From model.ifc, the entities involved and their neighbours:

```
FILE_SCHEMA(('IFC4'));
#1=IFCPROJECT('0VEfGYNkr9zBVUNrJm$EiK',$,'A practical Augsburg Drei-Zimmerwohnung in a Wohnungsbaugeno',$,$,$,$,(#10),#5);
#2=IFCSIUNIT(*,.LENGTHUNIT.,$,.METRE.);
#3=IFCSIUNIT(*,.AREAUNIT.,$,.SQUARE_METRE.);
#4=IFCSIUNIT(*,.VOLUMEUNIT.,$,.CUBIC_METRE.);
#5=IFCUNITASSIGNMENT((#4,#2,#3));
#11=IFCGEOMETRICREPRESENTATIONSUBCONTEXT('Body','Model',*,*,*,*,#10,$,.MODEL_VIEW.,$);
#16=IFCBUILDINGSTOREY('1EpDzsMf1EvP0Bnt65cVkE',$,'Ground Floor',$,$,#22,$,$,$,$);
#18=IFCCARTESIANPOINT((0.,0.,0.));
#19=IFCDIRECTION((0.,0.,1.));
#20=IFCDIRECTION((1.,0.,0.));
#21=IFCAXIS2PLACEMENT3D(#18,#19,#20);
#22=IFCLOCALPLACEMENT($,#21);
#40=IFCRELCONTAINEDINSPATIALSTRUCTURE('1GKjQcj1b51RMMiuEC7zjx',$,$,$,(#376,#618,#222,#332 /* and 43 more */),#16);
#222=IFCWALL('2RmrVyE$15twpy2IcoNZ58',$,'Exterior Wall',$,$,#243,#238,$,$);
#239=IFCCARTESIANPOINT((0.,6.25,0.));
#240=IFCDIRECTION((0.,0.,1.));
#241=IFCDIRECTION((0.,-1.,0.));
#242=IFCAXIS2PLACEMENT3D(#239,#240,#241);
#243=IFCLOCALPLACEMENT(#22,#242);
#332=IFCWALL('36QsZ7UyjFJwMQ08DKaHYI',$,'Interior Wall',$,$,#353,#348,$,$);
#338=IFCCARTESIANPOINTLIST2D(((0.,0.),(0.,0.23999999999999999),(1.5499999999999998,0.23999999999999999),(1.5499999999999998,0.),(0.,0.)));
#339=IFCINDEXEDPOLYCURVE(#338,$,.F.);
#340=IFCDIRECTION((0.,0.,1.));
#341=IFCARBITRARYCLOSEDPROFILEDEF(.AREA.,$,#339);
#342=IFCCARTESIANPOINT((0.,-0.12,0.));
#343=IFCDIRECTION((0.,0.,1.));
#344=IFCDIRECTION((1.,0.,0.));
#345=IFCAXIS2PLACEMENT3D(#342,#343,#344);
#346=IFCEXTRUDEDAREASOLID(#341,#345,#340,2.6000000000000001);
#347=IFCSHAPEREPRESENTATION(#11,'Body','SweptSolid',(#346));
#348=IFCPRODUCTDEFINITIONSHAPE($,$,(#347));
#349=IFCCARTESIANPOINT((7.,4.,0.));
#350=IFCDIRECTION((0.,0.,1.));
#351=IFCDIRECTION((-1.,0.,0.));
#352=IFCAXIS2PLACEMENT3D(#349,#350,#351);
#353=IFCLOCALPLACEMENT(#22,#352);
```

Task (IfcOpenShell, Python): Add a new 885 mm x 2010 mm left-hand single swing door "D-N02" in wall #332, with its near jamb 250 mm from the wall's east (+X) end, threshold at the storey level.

```python
import numpy as np
import ifcopenshell
import ifcopenshell.api.feature
import ifcopenshell.api.geometry
import ifcopenshell.api.root
import ifcopenshell.api.spatial
import ifcopenshell.geom
import ifcopenshell.util.element
import ifcopenshell.util.placement
import ifcopenshell.util.representation
import ifcopenshell.util.shape
import ifcopenshell.util.unit

model = ifcopenshell.open("model.ifc")
unit_scale = ifcopenshell.util.unit.calculate_unit_scale(model)
settings = ifcopenshell.geom.settings()


def volume(element):
    """Net volume in cubic metres, openings subtracted."""
    shape = ifcopenshell.geom.create_shape(settings, element)
    return ifcopenshell.util.shape.get_volume(shape.geometry)


wall = model.by_guid("36QsZ7UyjFJwMQ08DKaHYI")
storey = ifcopenshell.util.element.get_container(wall, ifc_class="IfcBuildingStorey")
context = ifcopenshell.util.representation.get_context(model, "Model", "Body", "MODEL_VIEW")
before = volume(wall)

width, height, from_end, sill = 0.885, 2.01, 0.25, 0.0  # metres

# The wall runs along its own X axis, and the end named is its -X end.
wall_shape = ifcopenshell.geom.create_shape(settings, wall)
x, y, z = ifcopenshell.util.shape.get_vertices(wall_shape.geometry).T
start = x.min() + from_end
face, thickness = float(y.min()), float(y.max() - y.min())
wall_matrix = ifcopenshell.util.placement.get_local_placement(wall.ObjectPlacement)
level = ifcopenshell.util.placement.get_local_placement(storey.ObjectPlacement)[2, 3]


def in_wall(x, y):
    """Placement at x, y metres in the wall's axes, at sill height."""
    matrix = wall_matrix.copy()
    matrix[:, 3] = wall_matrix @ np.array([x / unit_scale, y / unit_scale, 0.0, 1.0])
    matrix[2, 3] = level + sill / unit_scale
    return matrix


# Opening: a box that overshoots both wall faces by 50 mm.
opening = ifcopenshell.api.root.create_entity(model, ifc_class="IfcOpeningElement", predefined_type="OPENING")
box = ifcopenshell.api.geometry.add_wall_representation(
    model, context=context, length=width, height=height, thickness=thickness + 0.1
)
ifcopenshell.api.geometry.assign_representation(model, product=opening, representation=box)
ifcopenshell.api.geometry.edit_object_placement(model, product=opening, matrix=in_wall(start, face - 0.05), is_si=False)
ifcopenshell.api.feature.add_feature(model, feature=opening, element=wall)

door = ifcopenshell.api.root.create_entity(model, ifc_class="IfcDoor", name="D-N02", predefined_type="DOOR")
door.OverallWidth, door.OverallHeight = width / unit_scale, height / unit_scale
door.OperationType = "SINGLE_SWING_LEFT"
body = ifcopenshell.api.geometry.add_door_representation(
    model,
    context=context,
    overall_width=door.OverallWidth,
    overall_height=door.OverallHeight,
    operation_type="SINGLE_SWING_LEFT",
    lining_properties={"LiningDepth": thickness / unit_scale, "ThresholdDepth": thickness / unit_scale},
)
ifcopenshell.api.geometry.assign_representation(model, product=door, representation=body)
ifcopenshell.api.spatial.assign_container(model, products=[door], relating_structure=storey)
ifcopenshell.api.feature.add_filling(model, opening=opening, element=door)

# The lining spans the wall, so the door starts at the wall face.
ifcopenshell.api.geometry.edit_object_placement(model, product=door, matrix=in_wall(start, face), is_si=False)

after = volume(wall)

print(f"wall volume {before:.3f} -> {after:.3f} m3")

model.write("model_rev.ifc")
```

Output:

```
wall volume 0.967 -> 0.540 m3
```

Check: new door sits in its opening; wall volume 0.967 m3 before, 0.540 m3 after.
